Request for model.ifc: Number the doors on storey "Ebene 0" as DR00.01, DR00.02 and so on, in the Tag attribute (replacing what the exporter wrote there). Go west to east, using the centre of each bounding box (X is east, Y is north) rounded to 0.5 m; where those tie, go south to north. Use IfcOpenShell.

First a look at what the model holds.

```python
import ifcopenshell
import ifcopenshell.util.element
import ifcopenshell.util.placement

model = ifcopenshell.open("model.ifc")
print(model.schema)
storey = next(s for s in model.by_type("IfcBuildingStorey") if s.Name == "Ebene 0")
doors = [e for e in ifcopenshell.util.element.get_decomposition(storey) if e.is_a("IfcDoor")]
for e in sorted(doors, key=lambda e: e.id()):
    origin = ifcopenshell.util.placement.get_local_placement(e.ObjectPlacement)[:3, 3]
    print(e.id(), e.Tag, e.Name, origin.round(2) + 0.0, sep=" | ")
```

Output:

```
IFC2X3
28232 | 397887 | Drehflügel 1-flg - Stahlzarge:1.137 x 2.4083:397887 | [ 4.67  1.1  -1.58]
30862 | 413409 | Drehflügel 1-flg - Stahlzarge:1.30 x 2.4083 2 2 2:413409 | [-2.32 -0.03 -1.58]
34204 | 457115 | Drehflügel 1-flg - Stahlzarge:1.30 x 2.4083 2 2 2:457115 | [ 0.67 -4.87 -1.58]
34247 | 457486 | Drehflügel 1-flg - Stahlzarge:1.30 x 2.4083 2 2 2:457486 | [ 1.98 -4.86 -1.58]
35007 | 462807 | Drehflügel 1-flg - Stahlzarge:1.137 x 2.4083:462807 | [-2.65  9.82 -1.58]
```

```python
import ifcopenshell
import ifcopenshell.geom
import ifcopenshell.util.element
import ifcopenshell.util.shape

model = ifcopenshell.open("model.ifc")
settings = ifcopenshell.geom.settings()
settings.set("use-world-coords", True)


def centre(element):
    shape = ifcopenshell.geom.create_shape(settings, element)
    return ifcopenshell.util.shape.get_bbox_centroid(shape.geometry)


storey = next(s for s in model.by_type("IfcBuildingStorey") if s.Name == "Ebene 0")
doors = [e for e in ifcopenshell.util.element.get_decomposition(storey) if e.is_a("IfcDoor")]

# Insertion points can sit at a corner or the storey origin, so sort by the geometry (in metres).
centres = {e: centre(e) for e in doors}
doors.sort(key=lambda e: (round(centres[e][0] / 0.5), centres[e][1]))

for i, e in enumerate(doors, start=1):
    number = f"DR00.{i:02d}"
    e.Tag = number
    print(e.id(), number)

model.write("model_updated.ifc")
```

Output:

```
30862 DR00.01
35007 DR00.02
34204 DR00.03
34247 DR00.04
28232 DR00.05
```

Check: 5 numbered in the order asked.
